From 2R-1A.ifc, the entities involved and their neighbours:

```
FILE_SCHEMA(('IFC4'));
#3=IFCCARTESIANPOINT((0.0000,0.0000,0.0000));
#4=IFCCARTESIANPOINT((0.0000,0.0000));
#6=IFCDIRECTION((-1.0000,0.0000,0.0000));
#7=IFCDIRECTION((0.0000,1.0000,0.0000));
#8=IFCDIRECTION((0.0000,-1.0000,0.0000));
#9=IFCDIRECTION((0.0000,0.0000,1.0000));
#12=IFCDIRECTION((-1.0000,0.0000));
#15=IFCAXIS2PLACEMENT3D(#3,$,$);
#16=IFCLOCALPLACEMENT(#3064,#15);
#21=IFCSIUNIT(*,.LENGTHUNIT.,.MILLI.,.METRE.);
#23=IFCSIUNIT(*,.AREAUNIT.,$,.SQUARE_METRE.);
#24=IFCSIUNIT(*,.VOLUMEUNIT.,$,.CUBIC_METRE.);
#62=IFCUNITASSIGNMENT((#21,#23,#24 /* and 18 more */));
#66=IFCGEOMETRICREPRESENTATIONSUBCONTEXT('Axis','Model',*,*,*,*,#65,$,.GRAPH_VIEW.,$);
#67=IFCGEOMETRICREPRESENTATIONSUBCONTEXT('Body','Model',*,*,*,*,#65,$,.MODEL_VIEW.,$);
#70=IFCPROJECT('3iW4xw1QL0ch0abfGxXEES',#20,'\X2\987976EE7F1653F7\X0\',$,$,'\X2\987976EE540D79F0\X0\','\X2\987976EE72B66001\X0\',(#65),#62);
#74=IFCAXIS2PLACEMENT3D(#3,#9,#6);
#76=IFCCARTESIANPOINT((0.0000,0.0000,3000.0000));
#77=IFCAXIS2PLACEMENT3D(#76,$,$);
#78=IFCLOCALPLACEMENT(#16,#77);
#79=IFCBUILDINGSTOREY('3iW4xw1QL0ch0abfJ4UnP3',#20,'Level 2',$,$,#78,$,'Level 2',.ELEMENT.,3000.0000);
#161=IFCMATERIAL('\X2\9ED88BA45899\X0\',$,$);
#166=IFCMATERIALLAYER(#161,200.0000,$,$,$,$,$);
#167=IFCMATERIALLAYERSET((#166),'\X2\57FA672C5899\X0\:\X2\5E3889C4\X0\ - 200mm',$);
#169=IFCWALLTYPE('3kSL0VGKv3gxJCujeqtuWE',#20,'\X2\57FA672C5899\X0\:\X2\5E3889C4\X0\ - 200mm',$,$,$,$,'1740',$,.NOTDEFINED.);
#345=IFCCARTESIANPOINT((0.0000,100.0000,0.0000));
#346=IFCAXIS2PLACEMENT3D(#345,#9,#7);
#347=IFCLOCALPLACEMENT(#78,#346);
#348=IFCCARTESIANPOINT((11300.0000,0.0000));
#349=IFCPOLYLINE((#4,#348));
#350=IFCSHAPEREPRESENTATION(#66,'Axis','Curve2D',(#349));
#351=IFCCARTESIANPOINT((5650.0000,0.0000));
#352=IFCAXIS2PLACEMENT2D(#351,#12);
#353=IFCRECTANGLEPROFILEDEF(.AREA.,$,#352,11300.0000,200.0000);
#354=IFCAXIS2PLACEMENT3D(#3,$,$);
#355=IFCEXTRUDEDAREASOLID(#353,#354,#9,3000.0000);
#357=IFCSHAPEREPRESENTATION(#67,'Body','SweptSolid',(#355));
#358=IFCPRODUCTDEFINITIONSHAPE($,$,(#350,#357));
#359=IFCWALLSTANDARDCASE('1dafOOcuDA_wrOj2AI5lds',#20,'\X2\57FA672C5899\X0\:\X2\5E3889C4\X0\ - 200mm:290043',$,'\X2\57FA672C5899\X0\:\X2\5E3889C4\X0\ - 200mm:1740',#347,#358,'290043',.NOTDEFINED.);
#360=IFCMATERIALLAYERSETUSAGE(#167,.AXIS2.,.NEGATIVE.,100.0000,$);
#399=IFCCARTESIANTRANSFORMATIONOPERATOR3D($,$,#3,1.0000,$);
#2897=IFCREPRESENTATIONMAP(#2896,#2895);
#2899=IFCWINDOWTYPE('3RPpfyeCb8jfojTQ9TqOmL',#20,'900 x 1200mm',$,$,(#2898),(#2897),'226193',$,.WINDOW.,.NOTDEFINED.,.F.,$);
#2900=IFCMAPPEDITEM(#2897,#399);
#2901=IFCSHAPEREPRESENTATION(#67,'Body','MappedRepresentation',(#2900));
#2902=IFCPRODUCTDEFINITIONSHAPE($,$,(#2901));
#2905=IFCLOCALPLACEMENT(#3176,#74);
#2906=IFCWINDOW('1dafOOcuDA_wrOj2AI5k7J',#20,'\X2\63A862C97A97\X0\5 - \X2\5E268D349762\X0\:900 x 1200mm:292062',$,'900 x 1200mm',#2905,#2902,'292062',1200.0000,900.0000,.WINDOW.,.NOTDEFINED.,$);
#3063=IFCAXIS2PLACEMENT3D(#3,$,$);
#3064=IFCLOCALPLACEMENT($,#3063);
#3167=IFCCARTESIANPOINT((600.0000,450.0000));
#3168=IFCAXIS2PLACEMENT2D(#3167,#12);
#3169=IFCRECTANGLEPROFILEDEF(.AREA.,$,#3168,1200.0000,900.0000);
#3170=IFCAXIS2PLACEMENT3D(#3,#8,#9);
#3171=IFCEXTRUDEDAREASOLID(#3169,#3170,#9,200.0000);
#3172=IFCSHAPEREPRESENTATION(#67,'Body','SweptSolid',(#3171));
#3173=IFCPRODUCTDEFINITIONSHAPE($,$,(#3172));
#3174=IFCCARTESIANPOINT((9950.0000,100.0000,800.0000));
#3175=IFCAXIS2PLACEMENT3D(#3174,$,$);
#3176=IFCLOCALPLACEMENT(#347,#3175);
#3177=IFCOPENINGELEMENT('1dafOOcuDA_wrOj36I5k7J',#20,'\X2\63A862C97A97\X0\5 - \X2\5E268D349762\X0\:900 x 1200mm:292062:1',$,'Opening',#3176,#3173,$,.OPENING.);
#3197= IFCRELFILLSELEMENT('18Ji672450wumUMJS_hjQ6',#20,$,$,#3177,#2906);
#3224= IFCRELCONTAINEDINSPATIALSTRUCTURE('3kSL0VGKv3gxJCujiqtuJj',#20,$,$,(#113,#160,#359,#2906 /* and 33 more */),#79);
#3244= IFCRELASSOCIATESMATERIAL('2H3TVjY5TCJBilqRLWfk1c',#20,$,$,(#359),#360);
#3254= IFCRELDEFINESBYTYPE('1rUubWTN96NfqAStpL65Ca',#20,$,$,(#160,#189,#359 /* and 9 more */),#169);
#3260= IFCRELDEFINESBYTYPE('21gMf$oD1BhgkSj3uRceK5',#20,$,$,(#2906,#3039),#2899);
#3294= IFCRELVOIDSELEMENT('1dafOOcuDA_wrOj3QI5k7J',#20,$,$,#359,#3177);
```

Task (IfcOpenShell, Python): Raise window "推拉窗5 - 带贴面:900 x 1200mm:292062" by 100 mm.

```python
import numpy as np
import ifcopenshell
import ifcopenshell.api.geometry
import ifcopenshell.util.placement
import ifcopenshell.util.unit

model = ifcopenshell.open("2R-1A.ifc")
unit_scale = ifcopenshell.util.unit.calculate_unit_scale(model)

window = model.by_guid("1dafOOcuDA_wrOj2AI5k7J")
opening = window.FillsVoids[0].RelatingOpeningElement
dz = 0.1 / unit_scale

shift = np.array([0.0, 0.0, dz])
# The window is placed relative to its opening, so it follows when the opening moves.
matrix = ifcopenshell.util.placement.get_local_placement(opening.ObjectPlacement)
matrix[:3, 3] += shift
ifcopenshell.api.geometry.edit_object_placement(
    model, product=opening, matrix=matrix, is_si=False, should_transform_children=True
)

print(f"moved by {dz * unit_scale:+.3f} m")

model.write("2R-1A_edited.ifc")
```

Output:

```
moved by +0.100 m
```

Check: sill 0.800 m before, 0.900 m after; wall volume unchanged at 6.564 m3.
